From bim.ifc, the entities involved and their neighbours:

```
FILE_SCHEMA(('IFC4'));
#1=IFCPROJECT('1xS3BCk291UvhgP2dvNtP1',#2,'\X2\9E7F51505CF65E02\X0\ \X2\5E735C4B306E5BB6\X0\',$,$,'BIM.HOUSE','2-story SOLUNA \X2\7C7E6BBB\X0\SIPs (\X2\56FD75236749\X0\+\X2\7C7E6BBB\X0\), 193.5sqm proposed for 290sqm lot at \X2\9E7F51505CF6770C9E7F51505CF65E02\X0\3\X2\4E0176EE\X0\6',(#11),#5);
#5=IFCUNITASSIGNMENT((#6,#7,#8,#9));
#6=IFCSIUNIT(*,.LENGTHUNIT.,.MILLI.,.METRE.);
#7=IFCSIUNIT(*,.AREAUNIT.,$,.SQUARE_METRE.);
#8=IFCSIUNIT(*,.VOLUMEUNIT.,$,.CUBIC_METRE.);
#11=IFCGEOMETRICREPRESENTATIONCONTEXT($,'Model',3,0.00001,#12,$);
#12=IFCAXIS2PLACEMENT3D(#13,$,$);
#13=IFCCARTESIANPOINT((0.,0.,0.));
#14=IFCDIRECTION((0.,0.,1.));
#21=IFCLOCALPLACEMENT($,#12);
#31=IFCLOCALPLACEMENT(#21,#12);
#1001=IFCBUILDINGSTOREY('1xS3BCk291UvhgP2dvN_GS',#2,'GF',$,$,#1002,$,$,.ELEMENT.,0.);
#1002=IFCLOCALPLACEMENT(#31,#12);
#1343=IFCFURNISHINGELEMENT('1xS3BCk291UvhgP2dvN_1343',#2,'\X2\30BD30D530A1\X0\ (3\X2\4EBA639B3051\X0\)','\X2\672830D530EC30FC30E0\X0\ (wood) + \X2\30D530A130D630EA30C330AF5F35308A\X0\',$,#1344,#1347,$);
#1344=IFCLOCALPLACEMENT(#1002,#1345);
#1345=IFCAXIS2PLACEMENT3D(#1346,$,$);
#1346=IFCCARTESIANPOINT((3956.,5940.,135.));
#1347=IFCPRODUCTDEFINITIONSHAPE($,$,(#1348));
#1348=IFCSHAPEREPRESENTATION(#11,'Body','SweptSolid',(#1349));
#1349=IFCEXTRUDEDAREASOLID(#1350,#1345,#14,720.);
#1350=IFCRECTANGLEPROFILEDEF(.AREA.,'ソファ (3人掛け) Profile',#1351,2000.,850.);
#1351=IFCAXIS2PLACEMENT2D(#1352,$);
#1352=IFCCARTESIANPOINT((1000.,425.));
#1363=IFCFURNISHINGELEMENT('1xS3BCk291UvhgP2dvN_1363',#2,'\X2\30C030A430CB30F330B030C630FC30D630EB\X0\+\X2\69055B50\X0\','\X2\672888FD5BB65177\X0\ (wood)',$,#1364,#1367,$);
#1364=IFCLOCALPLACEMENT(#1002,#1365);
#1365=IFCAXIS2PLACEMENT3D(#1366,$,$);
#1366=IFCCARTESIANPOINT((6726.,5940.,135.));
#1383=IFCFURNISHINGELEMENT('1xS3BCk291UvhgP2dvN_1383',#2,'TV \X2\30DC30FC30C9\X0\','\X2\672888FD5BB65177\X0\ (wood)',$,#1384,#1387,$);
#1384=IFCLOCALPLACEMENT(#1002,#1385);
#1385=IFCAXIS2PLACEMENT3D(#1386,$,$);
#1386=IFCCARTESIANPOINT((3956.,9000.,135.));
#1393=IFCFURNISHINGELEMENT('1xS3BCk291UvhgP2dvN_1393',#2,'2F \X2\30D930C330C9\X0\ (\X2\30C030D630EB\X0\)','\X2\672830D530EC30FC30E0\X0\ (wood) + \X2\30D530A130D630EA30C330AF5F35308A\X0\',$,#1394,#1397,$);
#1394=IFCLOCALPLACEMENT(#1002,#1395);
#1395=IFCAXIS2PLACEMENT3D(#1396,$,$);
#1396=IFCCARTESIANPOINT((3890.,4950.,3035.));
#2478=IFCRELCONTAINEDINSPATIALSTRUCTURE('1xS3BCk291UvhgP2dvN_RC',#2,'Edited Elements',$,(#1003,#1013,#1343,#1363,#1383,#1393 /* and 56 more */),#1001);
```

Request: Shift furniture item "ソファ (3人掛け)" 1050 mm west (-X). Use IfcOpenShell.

```python
import ifcopenshell
import ifcopenshell.api.geometry
import ifcopenshell.util.placement
import ifcopenshell.util.unit

model = ifcopenshell.open("bim.ifc")
unit_scale = ifcopenshell.util.unit.calculate_unit_scale(model)

item = model.by_guid("1xS3BCk291UvhgP2dvN_1343")
matrix = ifcopenshell.util.placement.get_local_placement(item.ObjectPlacement)
matrix[0, 3] -= 1.05 / unit_scale
ifcopenshell.api.geometry.edit_object_placement(model, product=item, matrix=matrix, is_si=False)

print(ifcopenshell.util.placement.get_local_placement(item.ObjectPlacement).round(3) + 0.0)

model.write("bim_rev.ifc")
```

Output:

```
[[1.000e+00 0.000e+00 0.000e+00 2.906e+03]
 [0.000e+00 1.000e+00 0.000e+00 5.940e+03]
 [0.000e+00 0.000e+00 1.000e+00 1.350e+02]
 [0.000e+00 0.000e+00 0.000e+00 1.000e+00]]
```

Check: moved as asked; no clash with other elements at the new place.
